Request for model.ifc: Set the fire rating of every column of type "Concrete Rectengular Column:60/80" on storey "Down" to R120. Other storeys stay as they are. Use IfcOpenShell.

First a look at what the model holds.

```python
import ifcopenshell
import ifcopenshell.util.element

model = ifcopenshell.open("model.ifc")
print(model.schema)
storey = next(s for s in model.by_type("IfcBuildingStorey") if s.Name == "Down")
columns = [e for e in ifcopenshell.util.element.get_decomposition(storey) if e.is_a("IfcColumn")]
seen = {}
for e in columns:
    element_type = ifcopenshell.util.element.get_type(e)
    key = (element_type.Name if element_type != e and element_type else None, ifcopenshell.util.element.get_pset(e, "Pset_ColumnCommon", "FireRating"))
    seen[key] = seen.get(key, 0) + 1
for (name, value), count in sorted(seen.items(), key=str):
    print(count, "x", name, "|", value)
```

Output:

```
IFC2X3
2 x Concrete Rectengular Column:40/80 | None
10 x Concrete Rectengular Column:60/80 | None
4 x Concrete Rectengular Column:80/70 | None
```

```python
import ifcopenshell
import ifcopenshell.api.pset
import ifcopenshell.util.element

model = ifcopenshell.open("model.ifc")

storey = next(s for s in model.by_type("IfcBuildingStorey") if s.Name == "Down")
columns = [e for e in ifcopenshell.util.element.get_decomposition(storey) if e.is_a("IfcColumn")]

count = 0
for e in columns:
    element_type = ifcopenshell.util.element.get_type(e)
    if element_type in (None, e) or element_type.Name != "Concrete Rectengular Column:60/80":
        continue
    # add_pset returns the element's existing set when there is one.
    pset = ifcopenshell.api.pset.add_pset(model, product=e, name="Pset_ColumnCommon")
    ifcopenshell.api.pset.edit_pset(model, pset=pset, properties={"FireRating": "R120"})
    count += 1

print(count, "columns updated")

model.write("model_updated.ifc")
```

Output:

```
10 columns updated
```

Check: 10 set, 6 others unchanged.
